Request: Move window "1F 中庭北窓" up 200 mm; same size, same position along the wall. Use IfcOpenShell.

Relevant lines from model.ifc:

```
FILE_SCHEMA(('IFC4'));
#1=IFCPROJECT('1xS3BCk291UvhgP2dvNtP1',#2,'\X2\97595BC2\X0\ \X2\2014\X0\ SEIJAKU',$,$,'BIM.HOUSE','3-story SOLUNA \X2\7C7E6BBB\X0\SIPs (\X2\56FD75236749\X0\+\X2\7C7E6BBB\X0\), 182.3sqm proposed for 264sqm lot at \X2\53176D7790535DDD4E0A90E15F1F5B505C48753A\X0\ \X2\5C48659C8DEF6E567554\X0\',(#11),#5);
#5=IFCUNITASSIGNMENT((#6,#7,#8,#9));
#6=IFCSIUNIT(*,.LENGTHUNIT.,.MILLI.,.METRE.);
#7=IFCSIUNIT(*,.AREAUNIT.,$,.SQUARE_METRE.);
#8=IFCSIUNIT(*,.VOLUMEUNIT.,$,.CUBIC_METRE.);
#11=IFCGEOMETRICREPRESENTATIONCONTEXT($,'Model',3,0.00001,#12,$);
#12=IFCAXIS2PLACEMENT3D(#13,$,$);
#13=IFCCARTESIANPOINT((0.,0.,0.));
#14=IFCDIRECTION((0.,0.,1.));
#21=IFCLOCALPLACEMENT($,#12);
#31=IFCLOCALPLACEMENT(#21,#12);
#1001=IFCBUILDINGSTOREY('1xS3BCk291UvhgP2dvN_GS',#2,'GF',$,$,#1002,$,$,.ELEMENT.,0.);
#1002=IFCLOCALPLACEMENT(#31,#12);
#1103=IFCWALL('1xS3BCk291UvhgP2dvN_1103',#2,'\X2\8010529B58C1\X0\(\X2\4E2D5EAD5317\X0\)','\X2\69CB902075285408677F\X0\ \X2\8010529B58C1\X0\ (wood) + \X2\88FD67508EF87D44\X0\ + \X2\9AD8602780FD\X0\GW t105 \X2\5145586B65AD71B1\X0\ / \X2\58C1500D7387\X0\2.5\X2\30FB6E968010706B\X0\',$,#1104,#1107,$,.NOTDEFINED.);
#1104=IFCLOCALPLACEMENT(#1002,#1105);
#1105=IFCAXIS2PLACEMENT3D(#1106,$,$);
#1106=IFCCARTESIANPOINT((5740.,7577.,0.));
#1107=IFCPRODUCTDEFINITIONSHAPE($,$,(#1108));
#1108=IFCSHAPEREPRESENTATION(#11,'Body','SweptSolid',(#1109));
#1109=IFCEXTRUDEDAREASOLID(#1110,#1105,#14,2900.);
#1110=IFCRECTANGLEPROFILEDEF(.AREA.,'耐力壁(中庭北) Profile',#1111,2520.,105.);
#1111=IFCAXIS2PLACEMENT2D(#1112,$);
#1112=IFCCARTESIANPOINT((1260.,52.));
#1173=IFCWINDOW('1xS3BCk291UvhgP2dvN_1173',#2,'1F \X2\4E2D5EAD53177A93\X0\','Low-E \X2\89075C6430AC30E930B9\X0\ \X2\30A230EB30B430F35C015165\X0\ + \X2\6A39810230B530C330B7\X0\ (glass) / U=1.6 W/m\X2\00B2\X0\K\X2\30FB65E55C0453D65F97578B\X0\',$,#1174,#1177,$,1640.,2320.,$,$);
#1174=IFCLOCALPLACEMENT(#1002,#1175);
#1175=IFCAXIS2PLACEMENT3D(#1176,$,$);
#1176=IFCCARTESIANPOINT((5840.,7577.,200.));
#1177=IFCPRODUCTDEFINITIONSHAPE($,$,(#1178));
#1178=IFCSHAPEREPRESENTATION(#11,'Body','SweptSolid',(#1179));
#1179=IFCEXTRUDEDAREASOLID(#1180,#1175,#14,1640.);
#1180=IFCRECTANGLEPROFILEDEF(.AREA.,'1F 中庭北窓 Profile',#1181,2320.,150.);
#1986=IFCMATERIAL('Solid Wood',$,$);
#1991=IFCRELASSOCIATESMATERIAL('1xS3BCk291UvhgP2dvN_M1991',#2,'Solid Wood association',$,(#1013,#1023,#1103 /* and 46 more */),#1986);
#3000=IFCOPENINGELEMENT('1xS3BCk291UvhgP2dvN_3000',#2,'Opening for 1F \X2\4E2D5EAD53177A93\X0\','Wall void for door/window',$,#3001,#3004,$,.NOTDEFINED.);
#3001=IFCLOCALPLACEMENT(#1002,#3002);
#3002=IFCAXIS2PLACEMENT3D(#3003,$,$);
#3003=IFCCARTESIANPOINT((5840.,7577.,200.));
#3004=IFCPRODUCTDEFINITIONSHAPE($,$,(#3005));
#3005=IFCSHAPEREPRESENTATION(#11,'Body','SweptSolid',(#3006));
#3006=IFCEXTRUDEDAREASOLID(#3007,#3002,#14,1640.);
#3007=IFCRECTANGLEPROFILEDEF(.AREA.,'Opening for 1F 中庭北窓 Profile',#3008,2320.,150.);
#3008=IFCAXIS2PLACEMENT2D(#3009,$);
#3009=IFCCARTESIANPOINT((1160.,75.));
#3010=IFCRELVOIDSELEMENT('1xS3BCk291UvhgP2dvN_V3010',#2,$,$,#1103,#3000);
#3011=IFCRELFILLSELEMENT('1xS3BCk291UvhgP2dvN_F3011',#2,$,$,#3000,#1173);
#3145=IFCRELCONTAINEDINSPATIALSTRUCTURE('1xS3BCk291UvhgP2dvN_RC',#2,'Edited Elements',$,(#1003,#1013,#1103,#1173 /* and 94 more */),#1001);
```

```python
import numpy as np
import ifcopenshell
import ifcopenshell.api.geometry
import ifcopenshell.util.placement
import ifcopenshell.util.unit

model = ifcopenshell.open("model.ifc")
unit_scale = ifcopenshell.util.unit.calculate_unit_scale(model)

window = model.by_guid("1xS3BCk291UvhgP2dvN_1173")
opening = window.FillsVoids[0].RelatingOpeningElement
dz = 200.0

shift = np.array([0.0, 0.0, dz])
# The window is not placed relative to its opening, so move both.
for product in (opening, window):
    matrix = ifcopenshell.util.placement.get_local_placement(product.ObjectPlacement)
    matrix[:3, 3] += shift
    ifcopenshell.api.geometry.edit_object_placement(model, product=product, matrix=matrix, is_si=False)

print(f"moved by {dz * unit_scale:+.3f} m")

model.write("model_edited.ifc")
```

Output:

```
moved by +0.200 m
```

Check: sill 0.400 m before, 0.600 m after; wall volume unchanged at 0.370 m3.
